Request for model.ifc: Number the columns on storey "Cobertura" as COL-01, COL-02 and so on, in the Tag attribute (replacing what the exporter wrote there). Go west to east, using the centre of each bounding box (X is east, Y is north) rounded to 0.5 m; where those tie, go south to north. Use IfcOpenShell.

First a look at what the model holds.

```python
import ifcopenshell
import ifcopenshell.util.element
import ifcopenshell.util.placement

model = ifcopenshell.open("model.ifc")
print(model.schema)
storey = next(s for s in model.by_type("IfcBuildingStorey") if s.Name == "Cobertura")
columns = [e for e in ifcopenshell.util.element.get_decomposition(storey) if e.is_a("IfcColumn")]
for e in sorted(columns, key=lambda e: e.id()):
    origin = ifcopenshell.util.placement.get_local_placement(e.ObjectPlacement)[:3, 3]
    print(e.id(), e.Tag, e.Name, origin.round(2) + 0.0, sep=" | ")
```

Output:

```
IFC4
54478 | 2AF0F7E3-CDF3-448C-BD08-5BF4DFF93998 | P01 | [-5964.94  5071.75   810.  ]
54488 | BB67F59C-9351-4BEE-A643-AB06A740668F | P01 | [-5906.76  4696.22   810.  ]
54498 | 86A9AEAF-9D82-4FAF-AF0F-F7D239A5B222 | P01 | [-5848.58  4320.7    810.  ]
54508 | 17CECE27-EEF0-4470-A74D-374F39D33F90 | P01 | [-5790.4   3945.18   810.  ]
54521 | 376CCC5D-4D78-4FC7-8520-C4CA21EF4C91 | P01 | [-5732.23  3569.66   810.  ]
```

```python
import ifcopenshell
import ifcopenshell.geom
import ifcopenshell.util.element
import ifcopenshell.util.shape

model = ifcopenshell.open("model.ifc")
settings = ifcopenshell.geom.settings()
settings.set("use-world-coords", True)


def centre(element):
    shape = ifcopenshell.geom.create_shape(settings, element)
    return ifcopenshell.util.shape.get_bbox_centroid(shape.geometry)


storey = next(s for s in model.by_type("IfcBuildingStorey") if s.Name == "Cobertura")
columns = [e for e in ifcopenshell.util.element.get_decomposition(storey) if e.is_a("IfcColumn")]

# Insertion points can sit at a corner or the storey origin, so sort by the geometry (in metres).
centres = {e: centre(e) for e in columns}
columns.sort(key=lambda e: (round(centres[e][0] / 0.5), centres[e][1]))

for i, e in enumerate(columns, start=1):
    number = f"COL-{i:02d}"
    e.Tag = number
    print(e.id(), number)

model.write("model_updated.ifc")
```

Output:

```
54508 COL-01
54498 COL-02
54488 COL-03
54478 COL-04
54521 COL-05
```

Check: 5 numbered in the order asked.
